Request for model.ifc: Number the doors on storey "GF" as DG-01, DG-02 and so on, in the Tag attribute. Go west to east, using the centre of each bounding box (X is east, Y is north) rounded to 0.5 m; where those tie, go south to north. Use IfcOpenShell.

First a look at what the model holds.

```python
import ifcopenshell
import ifcopenshell.util.element
import ifcopenshell.util.placement

model = ifcopenshell.open("model.ifc")
print(model.schema)
storey = next(s for s in model.by_type("IfcBuildingStorey") if s.Name == "GF")
doors = [e for e in ifcopenshell.util.element.get_decomposition(storey) if e.is_a("IfcDoor")]
for e in sorted(doors, key=lambda e: e.id()):
    origin = ifcopenshell.util.placement.get_local_placement(e.ObjectPlacement)[:3, 3]
    print(e.id(), e.Tag, e.Name, origin.round(2) + 0.0, sep=" | ")
```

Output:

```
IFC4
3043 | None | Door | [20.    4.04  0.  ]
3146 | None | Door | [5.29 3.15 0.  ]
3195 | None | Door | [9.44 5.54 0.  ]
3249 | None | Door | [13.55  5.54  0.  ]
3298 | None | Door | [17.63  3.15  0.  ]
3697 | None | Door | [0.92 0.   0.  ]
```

```python
import ifcopenshell
import ifcopenshell.geom
import ifcopenshell.util.element
import ifcopenshell.util.shape

model = ifcopenshell.open("model.ifc")
settings = ifcopenshell.geom.settings()
settings.set("use-world-coords", True)


def centre(element):
    shape = ifcopenshell.geom.create_shape(settings, element)
    return ifcopenshell.util.shape.get_bbox_centroid(shape.geometry)


storey = next(s for s in model.by_type("IfcBuildingStorey") if s.Name == "GF")
doors = [e for e in ifcopenshell.util.element.get_decomposition(storey) if e.is_a("IfcDoor")]

# Insertion points can sit at a corner or the storey origin, so sort by the geometry (in metres).
centres = {e: centre(e) for e in doors}
doors.sort(key=lambda e: (round(centres[e][0] / 0.5), centres[e][1]))

for i, e in enumerate(doors, start=1):
    number = f"DG-{i:02d}"
    e.Tag = number
    print(e.id(), number)

model.write("model_edited.ifc")
```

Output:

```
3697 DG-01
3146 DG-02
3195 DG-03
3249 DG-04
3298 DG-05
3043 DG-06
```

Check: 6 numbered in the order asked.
